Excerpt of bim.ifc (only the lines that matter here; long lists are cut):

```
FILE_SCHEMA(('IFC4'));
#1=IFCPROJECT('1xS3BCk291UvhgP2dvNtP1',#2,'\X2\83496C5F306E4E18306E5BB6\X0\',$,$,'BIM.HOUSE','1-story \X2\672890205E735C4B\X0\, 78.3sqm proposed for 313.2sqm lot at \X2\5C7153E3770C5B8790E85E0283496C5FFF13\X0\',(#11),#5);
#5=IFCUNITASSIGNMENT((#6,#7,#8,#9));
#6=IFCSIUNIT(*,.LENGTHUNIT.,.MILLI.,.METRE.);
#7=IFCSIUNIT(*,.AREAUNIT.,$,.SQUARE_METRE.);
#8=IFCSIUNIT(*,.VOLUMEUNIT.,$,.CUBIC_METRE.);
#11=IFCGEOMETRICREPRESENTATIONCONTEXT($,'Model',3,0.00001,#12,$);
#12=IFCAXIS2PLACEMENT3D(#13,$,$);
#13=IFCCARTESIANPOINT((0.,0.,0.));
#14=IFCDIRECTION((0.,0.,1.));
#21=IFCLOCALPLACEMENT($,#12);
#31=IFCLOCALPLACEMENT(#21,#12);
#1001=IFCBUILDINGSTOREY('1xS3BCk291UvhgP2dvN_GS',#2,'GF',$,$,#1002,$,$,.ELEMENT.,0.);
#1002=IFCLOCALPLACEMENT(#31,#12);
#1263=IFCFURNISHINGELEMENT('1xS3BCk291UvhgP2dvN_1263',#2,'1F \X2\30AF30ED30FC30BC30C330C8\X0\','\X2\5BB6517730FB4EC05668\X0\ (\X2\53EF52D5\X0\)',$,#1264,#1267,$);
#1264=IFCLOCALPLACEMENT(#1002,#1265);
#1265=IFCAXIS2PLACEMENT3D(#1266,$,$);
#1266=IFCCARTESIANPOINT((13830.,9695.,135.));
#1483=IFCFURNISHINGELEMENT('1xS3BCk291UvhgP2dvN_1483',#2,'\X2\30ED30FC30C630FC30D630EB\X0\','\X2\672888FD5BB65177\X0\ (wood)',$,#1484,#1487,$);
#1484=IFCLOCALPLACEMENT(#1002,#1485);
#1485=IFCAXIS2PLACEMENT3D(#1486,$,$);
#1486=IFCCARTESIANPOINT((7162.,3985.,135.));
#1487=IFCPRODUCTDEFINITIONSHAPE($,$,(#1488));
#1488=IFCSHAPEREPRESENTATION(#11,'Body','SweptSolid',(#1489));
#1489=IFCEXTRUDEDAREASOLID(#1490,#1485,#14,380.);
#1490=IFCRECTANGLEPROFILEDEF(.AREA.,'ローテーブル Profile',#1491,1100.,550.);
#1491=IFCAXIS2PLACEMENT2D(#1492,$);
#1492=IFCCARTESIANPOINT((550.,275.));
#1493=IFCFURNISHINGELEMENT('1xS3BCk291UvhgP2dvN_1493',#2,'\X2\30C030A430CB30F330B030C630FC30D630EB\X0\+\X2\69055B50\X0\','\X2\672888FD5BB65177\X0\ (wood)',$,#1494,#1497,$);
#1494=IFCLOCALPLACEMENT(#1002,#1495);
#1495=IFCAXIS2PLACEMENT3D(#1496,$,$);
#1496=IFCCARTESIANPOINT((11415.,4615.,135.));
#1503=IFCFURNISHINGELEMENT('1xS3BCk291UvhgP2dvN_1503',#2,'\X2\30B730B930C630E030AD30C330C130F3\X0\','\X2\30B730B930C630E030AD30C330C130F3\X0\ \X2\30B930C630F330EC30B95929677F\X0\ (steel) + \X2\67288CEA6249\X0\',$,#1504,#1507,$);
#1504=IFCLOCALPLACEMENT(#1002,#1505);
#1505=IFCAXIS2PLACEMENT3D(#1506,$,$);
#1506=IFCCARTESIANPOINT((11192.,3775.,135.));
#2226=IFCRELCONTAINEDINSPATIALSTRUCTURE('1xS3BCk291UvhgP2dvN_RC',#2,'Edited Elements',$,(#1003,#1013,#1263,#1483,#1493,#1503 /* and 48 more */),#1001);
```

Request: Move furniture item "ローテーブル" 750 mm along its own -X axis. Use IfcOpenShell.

```python
import ifcopenshell
import ifcopenshell.api.geometry
import ifcopenshell.util.placement

model = ifcopenshell.open("bim.ifc")

item = model.by_guid("1xS3BCk291UvhgP2dvN_1483")
matrix = ifcopenshell.util.placement.get_local_placement(item.ObjectPlacement)
matrix[:3, 3] -= matrix[:3, 0] * 750.0
ifcopenshell.api.geometry.edit_object_placement(model, product=item, matrix=matrix, is_si=False)

print(ifcopenshell.util.placement.get_local_placement(item.ObjectPlacement).round(3) + 0.0)

model.write("bim_edited.ifc")
```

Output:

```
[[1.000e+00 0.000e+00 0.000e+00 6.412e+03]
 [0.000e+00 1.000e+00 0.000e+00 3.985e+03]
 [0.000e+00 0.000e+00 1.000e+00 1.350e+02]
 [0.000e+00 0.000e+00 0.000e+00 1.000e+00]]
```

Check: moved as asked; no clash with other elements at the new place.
